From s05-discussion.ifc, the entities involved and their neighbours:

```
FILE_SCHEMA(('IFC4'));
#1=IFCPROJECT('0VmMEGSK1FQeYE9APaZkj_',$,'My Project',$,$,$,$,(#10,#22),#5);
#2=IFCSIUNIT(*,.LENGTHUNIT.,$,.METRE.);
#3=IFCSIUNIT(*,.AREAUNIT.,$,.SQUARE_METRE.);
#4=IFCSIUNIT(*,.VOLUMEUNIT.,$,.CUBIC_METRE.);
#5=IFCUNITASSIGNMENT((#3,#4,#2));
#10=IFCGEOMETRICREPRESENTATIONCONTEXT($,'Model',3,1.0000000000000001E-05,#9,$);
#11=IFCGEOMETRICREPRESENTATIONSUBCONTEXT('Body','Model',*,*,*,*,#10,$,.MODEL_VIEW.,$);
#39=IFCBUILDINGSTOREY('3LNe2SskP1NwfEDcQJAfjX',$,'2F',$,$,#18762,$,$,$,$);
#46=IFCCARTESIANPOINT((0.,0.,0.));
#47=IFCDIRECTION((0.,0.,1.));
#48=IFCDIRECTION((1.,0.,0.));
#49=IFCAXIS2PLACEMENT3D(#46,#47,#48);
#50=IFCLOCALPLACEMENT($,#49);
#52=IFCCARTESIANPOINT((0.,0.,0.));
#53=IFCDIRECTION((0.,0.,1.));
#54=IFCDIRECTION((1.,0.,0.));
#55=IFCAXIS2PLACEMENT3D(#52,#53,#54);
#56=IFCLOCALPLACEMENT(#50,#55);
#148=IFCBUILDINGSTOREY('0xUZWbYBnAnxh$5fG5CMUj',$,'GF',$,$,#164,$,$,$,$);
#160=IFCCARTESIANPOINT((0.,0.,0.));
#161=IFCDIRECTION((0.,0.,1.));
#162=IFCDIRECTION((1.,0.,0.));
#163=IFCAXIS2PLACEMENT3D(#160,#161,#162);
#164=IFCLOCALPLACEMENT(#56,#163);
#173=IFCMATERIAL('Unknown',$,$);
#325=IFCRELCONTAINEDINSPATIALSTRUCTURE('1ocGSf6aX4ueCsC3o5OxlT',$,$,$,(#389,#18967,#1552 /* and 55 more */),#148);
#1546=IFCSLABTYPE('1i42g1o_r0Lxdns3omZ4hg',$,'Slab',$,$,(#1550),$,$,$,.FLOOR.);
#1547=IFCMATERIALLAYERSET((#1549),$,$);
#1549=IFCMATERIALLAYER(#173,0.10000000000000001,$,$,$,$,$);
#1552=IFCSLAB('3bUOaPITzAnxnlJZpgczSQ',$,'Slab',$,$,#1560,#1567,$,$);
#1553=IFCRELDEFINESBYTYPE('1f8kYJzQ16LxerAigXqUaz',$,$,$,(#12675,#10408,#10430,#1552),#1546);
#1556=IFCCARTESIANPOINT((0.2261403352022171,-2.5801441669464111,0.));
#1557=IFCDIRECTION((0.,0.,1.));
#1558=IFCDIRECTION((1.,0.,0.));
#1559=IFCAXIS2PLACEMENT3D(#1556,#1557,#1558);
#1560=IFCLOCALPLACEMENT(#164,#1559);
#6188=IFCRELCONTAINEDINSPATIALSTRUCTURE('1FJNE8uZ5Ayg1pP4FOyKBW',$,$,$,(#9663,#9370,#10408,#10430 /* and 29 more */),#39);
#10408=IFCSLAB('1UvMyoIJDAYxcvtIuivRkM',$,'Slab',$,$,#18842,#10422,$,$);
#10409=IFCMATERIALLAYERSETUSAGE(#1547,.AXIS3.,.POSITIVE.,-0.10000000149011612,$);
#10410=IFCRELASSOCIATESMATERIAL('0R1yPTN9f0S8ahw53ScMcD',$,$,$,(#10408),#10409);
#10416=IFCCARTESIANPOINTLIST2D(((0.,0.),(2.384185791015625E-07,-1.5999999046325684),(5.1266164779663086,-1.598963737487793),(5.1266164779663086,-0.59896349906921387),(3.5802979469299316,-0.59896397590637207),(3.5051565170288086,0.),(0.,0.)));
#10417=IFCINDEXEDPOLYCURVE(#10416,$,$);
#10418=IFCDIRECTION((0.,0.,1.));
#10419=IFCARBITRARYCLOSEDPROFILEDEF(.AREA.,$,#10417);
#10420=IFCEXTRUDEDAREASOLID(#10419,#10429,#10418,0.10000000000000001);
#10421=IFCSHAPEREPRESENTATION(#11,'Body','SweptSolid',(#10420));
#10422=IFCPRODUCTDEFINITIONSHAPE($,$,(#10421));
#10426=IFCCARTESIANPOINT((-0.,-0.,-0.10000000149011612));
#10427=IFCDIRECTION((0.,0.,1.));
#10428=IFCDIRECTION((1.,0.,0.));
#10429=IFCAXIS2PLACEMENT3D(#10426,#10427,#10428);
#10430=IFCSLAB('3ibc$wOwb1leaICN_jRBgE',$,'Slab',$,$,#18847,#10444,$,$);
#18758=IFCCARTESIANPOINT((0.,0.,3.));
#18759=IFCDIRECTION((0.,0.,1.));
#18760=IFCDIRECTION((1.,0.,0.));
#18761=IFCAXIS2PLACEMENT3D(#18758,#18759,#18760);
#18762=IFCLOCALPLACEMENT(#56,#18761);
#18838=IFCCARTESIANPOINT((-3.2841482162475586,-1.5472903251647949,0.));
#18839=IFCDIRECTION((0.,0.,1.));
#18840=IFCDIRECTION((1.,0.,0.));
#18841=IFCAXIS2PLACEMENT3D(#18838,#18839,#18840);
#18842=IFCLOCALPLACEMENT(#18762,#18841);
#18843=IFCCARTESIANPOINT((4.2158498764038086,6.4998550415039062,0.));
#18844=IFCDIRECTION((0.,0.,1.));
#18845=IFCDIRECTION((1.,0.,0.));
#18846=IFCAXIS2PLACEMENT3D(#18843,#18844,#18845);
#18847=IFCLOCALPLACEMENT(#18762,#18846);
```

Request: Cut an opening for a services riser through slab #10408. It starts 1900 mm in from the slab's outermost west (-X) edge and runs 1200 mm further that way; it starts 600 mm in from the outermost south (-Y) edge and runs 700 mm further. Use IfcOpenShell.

```python
import numpy as np
import ifcopenshell
import ifcopenshell.api.feature
import ifcopenshell.api.geometry
import ifcopenshell.api.root
import ifcopenshell.geom
import ifcopenshell.util.placement
import ifcopenshell.util.representation
import ifcopenshell.util.shape
import ifcopenshell.util.unit

model = ifcopenshell.open("s05-discussion.ifc")
unit_scale = ifcopenshell.util.unit.calculate_unit_scale(model)
settings = ifcopenshell.geom.settings()


def volume(element):
    """Net volume in cubic metres, openings subtracted."""
    shape = ifcopenshell.geom.create_shape(settings, element)
    return ifcopenshell.util.shape.get_volume(shape.geometry)


slab = model.by_guid("1UvMyoIJDAYxcvtIuivRkM")
before = volume(slab)

# Extent in the slab's own axes, in metres. The edges named are its -X and -Y sides.
slab_shape = ifcopenshell.geom.create_shape(settings, slab)
vertices = ifcopenshell.util.shape.get_vertices(slab_shape.geometry)
x_min, y_min, bottom = vertices.min(axis=0)
top = vertices[:, 2].max()

opening = ifcopenshell.api.root.create_entity(model, ifc_class="IfcOpeningElement", name="Services riser opening", predefined_type="OPENING")
context = ifcopenshell.util.representation.get_context(model, "Model", "Body", "MODEL_VIEW")
width, depth = 1.2, 0.7
outline = [(0.0, 0.0), (width, 0.0), (width, depth), (0.0, depth), (0.0, 0.0)]
# Overshoot both faces by 50 mm so the cut is clean.
shape = ifcopenshell.api.geometry.add_slab_representation(
    model, context=context, depth=top - bottom + 0.1, polyline=outline
)
ifcopenshell.api.geometry.assign_representation(model, product=opening, representation=shape)

matrix = ifcopenshell.util.placement.get_local_placement(slab.ObjectPlacement)
matrix[:, 3] = matrix @ np.append(np.array([x_min + 1.9, y_min + 0.6, bottom - 0.05]) / unit_scale, 1.0)
ifcopenshell.api.geometry.edit_object_placement(model, product=opening, matrix=matrix, is_si=False)
ifcopenshell.api.feature.add_feature(model, feature=opening, element=slab)

after = volume(slab)

print(f"slab volume {before:.3f} -> {after:.3f} m3")

model.write("s05-discussion_edited.ifc")
```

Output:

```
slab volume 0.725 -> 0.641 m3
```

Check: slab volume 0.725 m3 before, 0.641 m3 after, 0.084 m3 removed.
